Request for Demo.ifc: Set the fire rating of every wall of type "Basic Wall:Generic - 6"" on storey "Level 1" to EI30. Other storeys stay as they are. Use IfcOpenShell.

First a look at what the model holds.

```python
import ifcopenshell
import ifcopenshell.util.element

model = ifcopenshell.open("Demo.ifc")
print(model.schema)
storey = next(s for s in model.by_type("IfcBuildingStorey") if s.Name == "Level 1")
walls = [e for e in ifcopenshell.util.element.get_decomposition(storey) if e.is_a("IfcWall")]
seen = {}
for e in walls:
    element_type = ifcopenshell.util.element.get_type(e)
    key = (element_type.Name if element_type != e and element_type else None, ifcopenshell.util.element.get_pset(e, "Pset_WallCommon", "FireRating"))
    seen[key] = seen.get(key, 0) + 1
for (name, value), count in sorted(seen.items(), key=str):
    print(count, "x", name, "|", value)
```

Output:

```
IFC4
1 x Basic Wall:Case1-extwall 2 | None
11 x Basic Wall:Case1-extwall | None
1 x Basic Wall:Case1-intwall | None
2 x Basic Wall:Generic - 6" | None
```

```python
import ifcopenshell
import ifcopenshell.api.pset
import ifcopenshell.util.element

model = ifcopenshell.open("Demo.ifc")

storey = next(s for s in model.by_type("IfcBuildingStorey") if s.Name == "Level 1")
walls = [e for e in ifcopenshell.util.element.get_decomposition(storey) if e.is_a("IfcWall")]

count = 0
for e in walls:
    element_type = ifcopenshell.util.element.get_type(e)
    if element_type in (None, e) or element_type.Name != 'Basic Wall:Generic - 6"':
        continue
    # add_pset returns the element's existing set when there is one.
    pset = ifcopenshell.api.pset.add_pset(model, product=e, name="Pset_WallCommon")
    ifcopenshell.api.pset.edit_pset(model, pset=pset, properties={"FireRating": "EI30"})
    count += 1

print(count, "walls updated")

model.write("Demo-out.ifc")
```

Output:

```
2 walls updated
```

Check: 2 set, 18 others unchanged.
